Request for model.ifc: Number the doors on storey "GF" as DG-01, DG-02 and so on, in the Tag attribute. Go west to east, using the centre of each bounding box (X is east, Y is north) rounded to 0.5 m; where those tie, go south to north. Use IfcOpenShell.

First a look at what the model holds.

```python
import ifcopenshell
import ifcopenshell.util.element
import ifcopenshell.util.placement

model = ifcopenshell.open("model.ifc")
print(model.schema)
storey = next(s for s in model.by_type("IfcBuildingStorey") if s.Name == "GF")
doors = [e for e in ifcopenshell.util.element.get_decomposition(storey) if e.is_a("IfcDoor")]
for e in sorted(doors, key=lambda e: e.id()):
    origin = ifcopenshell.util.placement.get_local_placement(e.ObjectPlacement)[:3, 3]
    print(e.id(), e.Tag, e.Name, origin.round(2) + 0.0, sep=" | ")
```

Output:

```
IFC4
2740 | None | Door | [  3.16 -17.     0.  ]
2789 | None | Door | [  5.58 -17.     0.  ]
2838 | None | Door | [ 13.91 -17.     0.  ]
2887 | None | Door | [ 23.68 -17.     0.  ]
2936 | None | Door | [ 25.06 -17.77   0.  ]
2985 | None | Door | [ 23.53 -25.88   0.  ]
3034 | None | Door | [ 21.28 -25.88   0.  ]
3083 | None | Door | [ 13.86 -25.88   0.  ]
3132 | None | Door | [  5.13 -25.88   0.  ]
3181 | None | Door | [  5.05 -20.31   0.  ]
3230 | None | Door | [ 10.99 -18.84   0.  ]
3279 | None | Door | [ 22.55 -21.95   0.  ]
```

```python
import ifcopenshell
import ifcopenshell.geom
import ifcopenshell.util.element
import ifcopenshell.util.shape

model = ifcopenshell.open("model.ifc")
settings = ifcopenshell.geom.settings()
settings.set("use-world-coords", True)


def centre(element):
    shape = ifcopenshell.geom.create_shape(settings, element)
    return ifcopenshell.util.shape.get_bbox_centroid(shape.geometry)


storey = next(s for s in model.by_type("IfcBuildingStorey") if s.Name == "GF")
doors = [e for e in ifcopenshell.util.element.get_decomposition(storey) if e.is_a("IfcDoor")]

# Insertion points can sit at a corner or the storey origin, so sort by the geometry (in metres).
centres = {e: centre(e) for e in doors}
doors.sort(key=lambda e: (round(centres[e][0] / 0.5), centres[e][1]))

for i, e in enumerate(doors, start=1):
    number = f"DG-{i:02d}"
    e.Tag = number
    print(e.id(), number)

model.write("model_rev.ifc")
```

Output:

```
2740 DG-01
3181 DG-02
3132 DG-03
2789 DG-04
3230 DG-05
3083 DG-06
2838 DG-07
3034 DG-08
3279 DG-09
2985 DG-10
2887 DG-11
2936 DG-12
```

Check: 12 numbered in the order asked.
